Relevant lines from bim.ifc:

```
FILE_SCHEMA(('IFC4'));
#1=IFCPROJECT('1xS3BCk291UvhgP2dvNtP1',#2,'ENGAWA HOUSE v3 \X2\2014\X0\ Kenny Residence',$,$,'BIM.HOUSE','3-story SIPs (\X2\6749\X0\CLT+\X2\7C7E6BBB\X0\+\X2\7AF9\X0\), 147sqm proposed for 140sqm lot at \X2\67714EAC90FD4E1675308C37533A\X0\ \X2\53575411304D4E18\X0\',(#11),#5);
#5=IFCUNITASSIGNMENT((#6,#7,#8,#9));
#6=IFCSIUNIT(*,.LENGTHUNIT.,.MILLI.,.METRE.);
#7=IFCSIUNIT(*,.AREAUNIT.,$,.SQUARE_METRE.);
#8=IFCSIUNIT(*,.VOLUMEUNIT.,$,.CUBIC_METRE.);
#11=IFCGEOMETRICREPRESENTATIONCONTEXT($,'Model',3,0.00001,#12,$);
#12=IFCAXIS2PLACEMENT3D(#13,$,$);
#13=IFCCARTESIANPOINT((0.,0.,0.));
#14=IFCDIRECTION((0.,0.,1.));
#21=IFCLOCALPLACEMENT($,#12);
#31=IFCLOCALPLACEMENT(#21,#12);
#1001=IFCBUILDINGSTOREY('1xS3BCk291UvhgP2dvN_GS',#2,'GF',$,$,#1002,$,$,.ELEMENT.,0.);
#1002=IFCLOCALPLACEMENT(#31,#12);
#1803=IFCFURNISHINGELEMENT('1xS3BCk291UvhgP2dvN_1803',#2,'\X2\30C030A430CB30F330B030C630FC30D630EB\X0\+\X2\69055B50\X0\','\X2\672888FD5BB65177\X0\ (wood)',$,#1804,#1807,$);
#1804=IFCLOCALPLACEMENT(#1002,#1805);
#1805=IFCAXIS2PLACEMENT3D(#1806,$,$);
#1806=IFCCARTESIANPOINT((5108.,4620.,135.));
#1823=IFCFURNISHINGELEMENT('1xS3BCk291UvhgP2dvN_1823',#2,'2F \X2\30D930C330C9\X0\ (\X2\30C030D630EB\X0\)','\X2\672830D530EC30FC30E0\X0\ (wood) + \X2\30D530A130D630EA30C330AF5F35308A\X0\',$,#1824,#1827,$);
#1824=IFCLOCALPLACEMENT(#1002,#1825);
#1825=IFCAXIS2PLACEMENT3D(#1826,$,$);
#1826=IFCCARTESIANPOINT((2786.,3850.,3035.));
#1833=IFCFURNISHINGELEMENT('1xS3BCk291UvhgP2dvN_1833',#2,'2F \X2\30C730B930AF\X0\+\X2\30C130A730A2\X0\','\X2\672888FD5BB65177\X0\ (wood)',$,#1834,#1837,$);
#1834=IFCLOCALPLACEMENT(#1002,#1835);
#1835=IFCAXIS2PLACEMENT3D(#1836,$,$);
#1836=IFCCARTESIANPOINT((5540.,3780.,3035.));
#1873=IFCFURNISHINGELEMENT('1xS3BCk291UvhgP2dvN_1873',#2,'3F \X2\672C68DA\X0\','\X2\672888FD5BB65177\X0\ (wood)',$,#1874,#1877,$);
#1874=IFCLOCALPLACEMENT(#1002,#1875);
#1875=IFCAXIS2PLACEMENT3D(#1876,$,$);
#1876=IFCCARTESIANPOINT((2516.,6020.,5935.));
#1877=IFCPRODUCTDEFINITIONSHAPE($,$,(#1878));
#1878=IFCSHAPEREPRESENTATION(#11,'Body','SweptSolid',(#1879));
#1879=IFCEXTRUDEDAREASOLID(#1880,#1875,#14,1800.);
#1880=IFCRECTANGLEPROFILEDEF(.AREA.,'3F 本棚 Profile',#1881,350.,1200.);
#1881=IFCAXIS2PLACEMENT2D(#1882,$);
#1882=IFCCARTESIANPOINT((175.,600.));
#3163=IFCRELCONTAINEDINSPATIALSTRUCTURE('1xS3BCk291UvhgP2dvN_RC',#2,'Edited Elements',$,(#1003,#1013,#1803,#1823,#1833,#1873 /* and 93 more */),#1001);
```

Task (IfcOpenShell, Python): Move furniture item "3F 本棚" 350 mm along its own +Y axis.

```python
import ifcopenshell
import ifcopenshell.api.geometry
import ifcopenshell.util.placement
import ifcopenshell.util.unit

model = ifcopenshell.open("bim.ifc")
unit_scale = ifcopenshell.util.unit.calculate_unit_scale(model)

item = model.by_guid("1xS3BCk291UvhgP2dvN_1873")
matrix = ifcopenshell.util.placement.get_local_placement(item.ObjectPlacement)
matrix[:3, 3] += matrix[:3, 1] * 0.35 / unit_scale
ifcopenshell.api.geometry.edit_object_placement(model, product=item, matrix=matrix, is_si=False)

print(ifcopenshell.util.placement.get_local_placement(item.ObjectPlacement).round(3) + 0.0)

model.write("bim-out.ifc")
```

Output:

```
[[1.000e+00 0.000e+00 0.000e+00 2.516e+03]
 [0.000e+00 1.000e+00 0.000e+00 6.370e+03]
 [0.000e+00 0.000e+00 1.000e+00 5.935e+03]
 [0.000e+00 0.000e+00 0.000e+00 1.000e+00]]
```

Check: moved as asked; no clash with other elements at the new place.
